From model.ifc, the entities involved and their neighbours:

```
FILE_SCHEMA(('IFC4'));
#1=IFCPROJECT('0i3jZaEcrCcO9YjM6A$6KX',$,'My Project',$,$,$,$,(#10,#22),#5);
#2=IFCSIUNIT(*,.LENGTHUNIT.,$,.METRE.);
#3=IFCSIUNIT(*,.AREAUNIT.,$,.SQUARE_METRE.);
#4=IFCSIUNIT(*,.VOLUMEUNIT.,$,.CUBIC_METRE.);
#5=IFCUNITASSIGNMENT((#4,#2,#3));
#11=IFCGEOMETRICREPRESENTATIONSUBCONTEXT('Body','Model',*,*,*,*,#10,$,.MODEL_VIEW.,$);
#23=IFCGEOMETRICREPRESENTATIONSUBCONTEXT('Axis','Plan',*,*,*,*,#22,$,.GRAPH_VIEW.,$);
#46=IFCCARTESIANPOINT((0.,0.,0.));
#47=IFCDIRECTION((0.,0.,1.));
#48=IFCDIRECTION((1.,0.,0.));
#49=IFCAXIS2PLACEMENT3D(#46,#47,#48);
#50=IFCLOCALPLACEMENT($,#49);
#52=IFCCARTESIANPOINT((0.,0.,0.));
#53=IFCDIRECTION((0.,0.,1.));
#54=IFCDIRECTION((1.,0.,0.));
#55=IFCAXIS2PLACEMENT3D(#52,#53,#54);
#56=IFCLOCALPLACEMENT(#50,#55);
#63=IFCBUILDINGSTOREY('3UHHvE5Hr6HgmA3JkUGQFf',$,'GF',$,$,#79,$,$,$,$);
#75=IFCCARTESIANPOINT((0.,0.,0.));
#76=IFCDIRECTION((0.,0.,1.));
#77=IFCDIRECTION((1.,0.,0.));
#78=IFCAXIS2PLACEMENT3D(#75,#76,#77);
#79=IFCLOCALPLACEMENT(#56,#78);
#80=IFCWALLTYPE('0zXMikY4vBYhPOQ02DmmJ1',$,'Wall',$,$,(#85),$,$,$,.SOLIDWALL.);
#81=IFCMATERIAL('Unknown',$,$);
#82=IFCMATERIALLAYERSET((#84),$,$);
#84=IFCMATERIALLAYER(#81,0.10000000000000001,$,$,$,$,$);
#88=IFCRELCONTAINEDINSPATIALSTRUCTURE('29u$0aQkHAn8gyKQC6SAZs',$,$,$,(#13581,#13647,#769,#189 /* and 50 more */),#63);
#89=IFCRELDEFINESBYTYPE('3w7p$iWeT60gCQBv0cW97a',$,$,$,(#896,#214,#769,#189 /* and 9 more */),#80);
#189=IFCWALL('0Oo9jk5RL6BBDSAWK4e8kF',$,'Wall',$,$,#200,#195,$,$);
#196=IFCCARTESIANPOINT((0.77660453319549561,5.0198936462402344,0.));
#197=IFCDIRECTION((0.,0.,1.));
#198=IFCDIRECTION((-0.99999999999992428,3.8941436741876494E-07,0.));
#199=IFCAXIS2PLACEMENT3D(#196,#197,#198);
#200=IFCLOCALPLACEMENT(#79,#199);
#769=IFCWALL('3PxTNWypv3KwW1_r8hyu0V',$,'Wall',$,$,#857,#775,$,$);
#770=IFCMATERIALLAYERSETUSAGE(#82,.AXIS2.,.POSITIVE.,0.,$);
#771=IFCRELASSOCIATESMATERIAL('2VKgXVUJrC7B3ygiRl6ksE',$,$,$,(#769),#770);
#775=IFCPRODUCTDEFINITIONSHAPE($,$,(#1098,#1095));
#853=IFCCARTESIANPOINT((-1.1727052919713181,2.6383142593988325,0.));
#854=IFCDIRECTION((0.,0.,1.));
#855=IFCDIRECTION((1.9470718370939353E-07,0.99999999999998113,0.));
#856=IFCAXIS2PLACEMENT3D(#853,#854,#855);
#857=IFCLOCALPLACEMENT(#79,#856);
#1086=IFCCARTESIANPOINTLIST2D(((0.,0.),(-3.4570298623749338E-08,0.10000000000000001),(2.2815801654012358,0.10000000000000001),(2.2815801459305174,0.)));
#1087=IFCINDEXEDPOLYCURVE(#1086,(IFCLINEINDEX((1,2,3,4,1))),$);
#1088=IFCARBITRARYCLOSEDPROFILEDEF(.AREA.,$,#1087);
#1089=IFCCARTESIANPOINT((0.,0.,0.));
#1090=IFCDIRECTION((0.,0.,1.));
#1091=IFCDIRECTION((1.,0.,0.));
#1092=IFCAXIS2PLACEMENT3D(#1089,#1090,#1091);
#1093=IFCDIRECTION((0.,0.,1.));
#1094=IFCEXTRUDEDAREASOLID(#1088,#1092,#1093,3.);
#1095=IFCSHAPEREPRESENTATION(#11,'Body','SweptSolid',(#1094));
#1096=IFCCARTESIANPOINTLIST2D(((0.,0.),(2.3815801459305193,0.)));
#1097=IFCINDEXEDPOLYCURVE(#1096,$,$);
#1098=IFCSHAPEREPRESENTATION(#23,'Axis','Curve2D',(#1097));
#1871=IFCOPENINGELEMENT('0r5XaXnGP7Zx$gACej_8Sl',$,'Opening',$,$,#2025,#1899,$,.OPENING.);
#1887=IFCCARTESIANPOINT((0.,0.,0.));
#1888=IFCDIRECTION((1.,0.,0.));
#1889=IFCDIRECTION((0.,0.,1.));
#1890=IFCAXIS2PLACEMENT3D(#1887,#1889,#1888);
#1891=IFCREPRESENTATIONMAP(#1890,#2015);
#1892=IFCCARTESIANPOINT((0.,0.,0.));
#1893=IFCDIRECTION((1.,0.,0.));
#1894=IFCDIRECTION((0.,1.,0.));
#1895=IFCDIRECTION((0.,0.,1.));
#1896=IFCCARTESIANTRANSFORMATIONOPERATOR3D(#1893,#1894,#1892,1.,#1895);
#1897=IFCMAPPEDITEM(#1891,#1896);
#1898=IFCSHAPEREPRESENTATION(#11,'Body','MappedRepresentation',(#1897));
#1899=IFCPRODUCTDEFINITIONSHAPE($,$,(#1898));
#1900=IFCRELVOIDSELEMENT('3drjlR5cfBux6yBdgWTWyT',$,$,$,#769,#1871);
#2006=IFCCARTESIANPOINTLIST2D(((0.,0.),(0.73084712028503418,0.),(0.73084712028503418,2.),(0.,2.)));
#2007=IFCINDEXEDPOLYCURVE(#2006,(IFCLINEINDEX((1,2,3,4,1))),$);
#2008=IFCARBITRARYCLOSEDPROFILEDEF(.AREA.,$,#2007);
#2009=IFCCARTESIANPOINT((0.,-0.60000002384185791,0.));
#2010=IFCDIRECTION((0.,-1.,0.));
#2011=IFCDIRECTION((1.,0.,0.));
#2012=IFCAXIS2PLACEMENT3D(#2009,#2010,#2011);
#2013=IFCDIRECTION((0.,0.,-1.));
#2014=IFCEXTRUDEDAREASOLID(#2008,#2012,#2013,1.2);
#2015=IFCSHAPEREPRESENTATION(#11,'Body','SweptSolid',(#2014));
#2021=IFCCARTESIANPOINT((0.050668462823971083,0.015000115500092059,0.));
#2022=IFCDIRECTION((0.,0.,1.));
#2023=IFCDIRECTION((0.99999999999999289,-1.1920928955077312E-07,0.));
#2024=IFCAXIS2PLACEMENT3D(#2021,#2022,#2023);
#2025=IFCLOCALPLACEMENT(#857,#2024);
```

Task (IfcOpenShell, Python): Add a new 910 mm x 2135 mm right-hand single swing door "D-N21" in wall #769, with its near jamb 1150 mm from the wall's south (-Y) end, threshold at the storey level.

```python
import numpy as np
import ifcopenshell
import ifcopenshell.api.feature
import ifcopenshell.api.geometry
import ifcopenshell.api.root
import ifcopenshell.api.spatial
import ifcopenshell.geom
import ifcopenshell.util.element
import ifcopenshell.util.placement
import ifcopenshell.util.representation
import ifcopenshell.util.shape
import ifcopenshell.util.unit

model = ifcopenshell.open("model.ifc")
unit_scale = ifcopenshell.util.unit.calculate_unit_scale(model)
settings = ifcopenshell.geom.settings()


def volume(element):
    """Net volume in cubic metres, openings subtracted."""
    shape = ifcopenshell.geom.create_shape(settings, element)
    return ifcopenshell.util.shape.get_volume(shape.geometry)


wall = model.by_guid("3PxTNWypv3KwW1_r8hyu0V")
storey = ifcopenshell.util.element.get_container(wall, ifc_class="IfcBuildingStorey")
context = ifcopenshell.util.representation.get_context(model, "Model", "Body", "MODEL_VIEW")
before = volume(wall)

width, height, from_end, sill = 0.91, 2.135, 1.15, 0.0  # metres

# The wall runs along its own X axis, and the end named is its -X end.
wall_shape = ifcopenshell.geom.create_shape(settings, wall)
x, y, z = ifcopenshell.util.shape.get_vertices(wall_shape.geometry).T
start = x.min() + from_end
face, thickness = float(y.min()), float(y.max() - y.min())
wall_matrix = ifcopenshell.util.placement.get_local_placement(wall.ObjectPlacement)
level = ifcopenshell.util.placement.get_local_placement(storey.ObjectPlacement)[2, 3]


def in_wall(x, y):
    """Placement at x, y metres in the wall's axes, at sill height."""
    matrix = wall_matrix.copy()
    matrix[:, 3] = wall_matrix @ np.array([x / unit_scale, y / unit_scale, 0.0, 1.0])
    matrix[2, 3] = level + sill / unit_scale
    return matrix


# Opening: a box that overshoots both wall faces by 50 mm.
opening = ifcopenshell.api.root.create_entity(model, ifc_class="IfcOpeningElement", predefined_type="OPENING")
box = ifcopenshell.api.geometry.add_wall_representation(
    model, context=context, length=width, height=height, thickness=thickness + 0.1
)
ifcopenshell.api.geometry.assign_representation(model, product=opening, representation=box)
ifcopenshell.api.geometry.edit_object_placement(model, product=opening, matrix=in_wall(start, face - 0.05), is_si=False)
ifcopenshell.api.feature.add_feature(model, feature=opening, element=wall)

door = ifcopenshell.api.root.create_entity(model, ifc_class="IfcDoor", name="D-N21", predefined_type="DOOR")
door.OverallWidth, door.OverallHeight = width / unit_scale, height / unit_scale
door.OperationType = "SINGLE_SWING_RIGHT"
body = ifcopenshell.api.geometry.add_door_representation(
    model,
    context=context,
    overall_width=door.OverallWidth,
    overall_height=door.OverallHeight,
    operation_type="SINGLE_SWING_RIGHT",
    lining_properties={"LiningDepth": thickness / unit_scale, "ThresholdDepth": thickness / unit_scale},
)
ifcopenshell.api.geometry.assign_representation(model, product=door, representation=body)
ifcopenshell.api.spatial.assign_container(model, products=[door], relating_structure=storey)
ifcopenshell.api.feature.add_filling(model, opening=opening, element=door)

# The lining spans the wall, so the door starts at the wall face.
ifcopenshell.api.geometry.edit_object_placement(model, product=door, matrix=in_wall(start, face), is_si=False)

after = volume(wall)

print(f"wall volume {before:.3f} -> {after:.3f} m3")

model.write("model_v2.ifc")
```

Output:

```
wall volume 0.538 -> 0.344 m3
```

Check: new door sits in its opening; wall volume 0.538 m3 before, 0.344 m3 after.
